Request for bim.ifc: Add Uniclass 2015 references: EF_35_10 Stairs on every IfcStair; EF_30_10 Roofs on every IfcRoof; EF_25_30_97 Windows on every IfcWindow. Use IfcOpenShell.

First a look at what the model holds.

```python
import ifcopenshell

model = ifcopenshell.open("bim.ifc")
print(model.schema)
print("classifications:", [c.Name for c in model.by_type("IfcClassification")])
for ifc_class in ("IfcDoor", "IfcRoof", "IfcStair", "IfcWall", "IfcWindow"):
    print(ifc_class, len(model.by_type(ifc_class)))
```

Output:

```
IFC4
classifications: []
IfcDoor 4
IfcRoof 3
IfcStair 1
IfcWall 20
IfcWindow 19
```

```python
import ifcopenshell
import ifcopenshell.api.classification

model = ifcopenshell.open("bim.ifc")

system = ifcopenshell.api.classification.add_classification(model, classification="Uniclass 2015")

codes = {
    "IfcStair": ("EF_35_10", "Stairs"),
    "IfcRoof": ("EF_30_10", "Roofs"),
    "IfcWindow": ("EF_25_30_97", "Windows"),
}
for ifc_class, (code, name) in codes.items():
    products = model.by_type(ifc_class)
    ifcopenshell.api.classification.add_reference(
        model, products=products, classification=system, identification=code, name=name
    )
    print(code, len(products))

model.write("bim_edited.ifc")
```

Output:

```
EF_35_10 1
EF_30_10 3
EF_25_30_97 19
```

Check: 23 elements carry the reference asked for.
